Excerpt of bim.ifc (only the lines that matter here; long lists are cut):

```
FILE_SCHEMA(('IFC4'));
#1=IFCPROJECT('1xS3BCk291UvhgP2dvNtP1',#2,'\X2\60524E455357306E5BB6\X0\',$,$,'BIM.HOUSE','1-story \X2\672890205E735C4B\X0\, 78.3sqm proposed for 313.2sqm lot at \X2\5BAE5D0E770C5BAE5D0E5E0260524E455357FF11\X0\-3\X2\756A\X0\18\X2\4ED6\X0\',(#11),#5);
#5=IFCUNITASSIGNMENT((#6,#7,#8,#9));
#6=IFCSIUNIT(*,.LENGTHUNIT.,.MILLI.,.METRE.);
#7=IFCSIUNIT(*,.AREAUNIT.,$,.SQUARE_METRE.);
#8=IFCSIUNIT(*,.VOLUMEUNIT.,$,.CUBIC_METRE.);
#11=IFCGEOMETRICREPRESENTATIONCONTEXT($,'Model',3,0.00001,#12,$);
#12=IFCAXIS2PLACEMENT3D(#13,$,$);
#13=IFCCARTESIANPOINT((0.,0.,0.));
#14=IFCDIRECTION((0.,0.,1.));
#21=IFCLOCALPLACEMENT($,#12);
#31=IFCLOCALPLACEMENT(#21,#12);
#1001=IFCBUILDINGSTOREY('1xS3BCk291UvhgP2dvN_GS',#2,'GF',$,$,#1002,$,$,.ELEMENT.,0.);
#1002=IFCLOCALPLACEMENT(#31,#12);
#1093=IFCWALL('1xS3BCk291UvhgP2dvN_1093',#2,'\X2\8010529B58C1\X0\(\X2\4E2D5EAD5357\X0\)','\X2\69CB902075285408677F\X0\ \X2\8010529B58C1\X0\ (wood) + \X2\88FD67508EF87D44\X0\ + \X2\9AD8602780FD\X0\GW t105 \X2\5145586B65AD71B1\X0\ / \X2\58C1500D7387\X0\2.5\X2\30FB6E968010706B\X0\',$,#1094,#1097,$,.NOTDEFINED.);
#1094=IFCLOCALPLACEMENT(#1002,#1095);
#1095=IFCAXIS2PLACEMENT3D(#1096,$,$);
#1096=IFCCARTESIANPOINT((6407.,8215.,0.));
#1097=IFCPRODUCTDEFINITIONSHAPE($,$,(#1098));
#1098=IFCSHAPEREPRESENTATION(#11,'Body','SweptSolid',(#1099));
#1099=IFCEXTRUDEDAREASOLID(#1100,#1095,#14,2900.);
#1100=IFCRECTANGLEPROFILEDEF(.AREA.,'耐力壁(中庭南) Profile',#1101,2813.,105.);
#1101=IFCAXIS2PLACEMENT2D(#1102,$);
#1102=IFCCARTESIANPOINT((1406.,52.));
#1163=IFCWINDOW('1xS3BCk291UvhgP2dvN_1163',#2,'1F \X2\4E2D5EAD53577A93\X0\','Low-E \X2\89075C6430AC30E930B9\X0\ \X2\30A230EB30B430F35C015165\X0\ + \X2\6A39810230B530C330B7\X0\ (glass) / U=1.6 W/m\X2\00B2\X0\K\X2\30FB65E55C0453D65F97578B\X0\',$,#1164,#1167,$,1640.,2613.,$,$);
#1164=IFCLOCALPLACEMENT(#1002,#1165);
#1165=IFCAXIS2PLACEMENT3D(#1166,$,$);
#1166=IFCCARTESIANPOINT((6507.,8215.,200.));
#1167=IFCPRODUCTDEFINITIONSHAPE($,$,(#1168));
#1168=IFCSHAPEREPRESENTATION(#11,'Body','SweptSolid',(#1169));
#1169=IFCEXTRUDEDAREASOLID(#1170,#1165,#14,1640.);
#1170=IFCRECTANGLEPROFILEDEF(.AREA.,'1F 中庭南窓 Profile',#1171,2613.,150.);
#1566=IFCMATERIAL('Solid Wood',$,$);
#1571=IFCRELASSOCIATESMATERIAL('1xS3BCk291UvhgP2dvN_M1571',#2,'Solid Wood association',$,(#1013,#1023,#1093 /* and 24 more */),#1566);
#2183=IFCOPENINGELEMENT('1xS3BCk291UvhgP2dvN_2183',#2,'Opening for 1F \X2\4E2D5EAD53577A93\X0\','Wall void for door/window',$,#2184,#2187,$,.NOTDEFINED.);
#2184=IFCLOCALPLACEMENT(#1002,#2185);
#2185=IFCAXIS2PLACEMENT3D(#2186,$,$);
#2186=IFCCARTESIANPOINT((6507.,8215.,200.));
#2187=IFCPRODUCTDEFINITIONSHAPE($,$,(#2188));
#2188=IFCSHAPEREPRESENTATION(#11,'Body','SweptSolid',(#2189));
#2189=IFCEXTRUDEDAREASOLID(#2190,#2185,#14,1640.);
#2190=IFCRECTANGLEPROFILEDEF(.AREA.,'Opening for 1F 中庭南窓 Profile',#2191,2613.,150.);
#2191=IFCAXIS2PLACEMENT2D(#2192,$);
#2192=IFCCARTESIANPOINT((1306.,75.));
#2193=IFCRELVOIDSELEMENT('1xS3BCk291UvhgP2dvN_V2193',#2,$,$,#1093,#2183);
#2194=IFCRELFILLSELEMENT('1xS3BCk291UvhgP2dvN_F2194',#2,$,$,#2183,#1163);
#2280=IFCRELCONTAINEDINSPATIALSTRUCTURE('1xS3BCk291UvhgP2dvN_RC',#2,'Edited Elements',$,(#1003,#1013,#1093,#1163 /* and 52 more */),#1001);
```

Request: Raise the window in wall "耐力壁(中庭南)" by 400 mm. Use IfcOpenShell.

```python
import numpy as np
import ifcopenshell
import ifcopenshell.api.geometry
import ifcopenshell.util.placement
import ifcopenshell.util.unit

model = ifcopenshell.open("bim.ifc")
unit_scale = ifcopenshell.util.unit.calculate_unit_scale(model)

window = model.by_guid("1xS3BCk291UvhgP2dvN_1163")
opening = window.FillsVoids[0].RelatingOpeningElement
dz = 400.0

shift = np.array([0.0, 0.0, dz])
# The window is not placed relative to its opening, so move both.
for product in (opening, window):
    matrix = ifcopenshell.util.placement.get_local_placement(product.ObjectPlacement)
    matrix[:3, 3] += shift
    ifcopenshell.api.geometry.edit_object_placement(model, product=product, matrix=matrix, is_si=False)

print(f"moved by {dz * unit_scale:+.3f} m")

model.write("bim_edited.ifc")
```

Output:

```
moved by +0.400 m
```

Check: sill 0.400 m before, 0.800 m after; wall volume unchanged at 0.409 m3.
